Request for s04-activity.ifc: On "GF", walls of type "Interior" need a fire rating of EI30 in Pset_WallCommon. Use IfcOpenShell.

First a look at what the model holds.

```python
import ifcopenshell
import ifcopenshell.util.element

model = ifcopenshell.open("s04-activity.ifc")
print(model.schema)
storey = next(s for s in model.by_type("IfcBuildingStorey") if s.Name == "GF")
walls = [e for e in ifcopenshell.util.element.get_decomposition(storey) if e.is_a("IfcWall")]
seen = {}
for e in walls:
    element_type = ifcopenshell.util.element.get_type(e)
    key = (element_type.Name if element_type != e and element_type else None, ifcopenshell.util.element.get_pset(e, "Pset_WallCommon", "FireRating"))
    seen[key] = seen.get(key, 0) + 1
for (name, value), count in sorted(seen.items(), key=str):
    print(count, "x", name, "|", value)
```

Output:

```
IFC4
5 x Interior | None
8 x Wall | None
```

```python
import ifcopenshell
import ifcopenshell.api.pset
import ifcopenshell.util.element

model = ifcopenshell.open("s04-activity.ifc")

storey = next(s for s in model.by_type("IfcBuildingStorey") if s.Name == "GF")
walls = [e for e in ifcopenshell.util.element.get_decomposition(storey) if e.is_a("IfcWall")]

count = 0
for e in walls:
    element_type = ifcopenshell.util.element.get_type(e)
    if element_type in (None, e) or element_type.Name != "Interior":
        continue
    # add_pset returns the element's existing set when there is one.
    pset = ifcopenshell.api.pset.add_pset(model, product=e, name="Pset_WallCommon")
    ifcopenshell.api.pset.edit_pset(model, pset=pset, properties={"FireRating": "EI30"})
    count += 1

print(count, "walls updated")

model.write("s04-activity_v2.ifc")
```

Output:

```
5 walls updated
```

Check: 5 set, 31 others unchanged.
